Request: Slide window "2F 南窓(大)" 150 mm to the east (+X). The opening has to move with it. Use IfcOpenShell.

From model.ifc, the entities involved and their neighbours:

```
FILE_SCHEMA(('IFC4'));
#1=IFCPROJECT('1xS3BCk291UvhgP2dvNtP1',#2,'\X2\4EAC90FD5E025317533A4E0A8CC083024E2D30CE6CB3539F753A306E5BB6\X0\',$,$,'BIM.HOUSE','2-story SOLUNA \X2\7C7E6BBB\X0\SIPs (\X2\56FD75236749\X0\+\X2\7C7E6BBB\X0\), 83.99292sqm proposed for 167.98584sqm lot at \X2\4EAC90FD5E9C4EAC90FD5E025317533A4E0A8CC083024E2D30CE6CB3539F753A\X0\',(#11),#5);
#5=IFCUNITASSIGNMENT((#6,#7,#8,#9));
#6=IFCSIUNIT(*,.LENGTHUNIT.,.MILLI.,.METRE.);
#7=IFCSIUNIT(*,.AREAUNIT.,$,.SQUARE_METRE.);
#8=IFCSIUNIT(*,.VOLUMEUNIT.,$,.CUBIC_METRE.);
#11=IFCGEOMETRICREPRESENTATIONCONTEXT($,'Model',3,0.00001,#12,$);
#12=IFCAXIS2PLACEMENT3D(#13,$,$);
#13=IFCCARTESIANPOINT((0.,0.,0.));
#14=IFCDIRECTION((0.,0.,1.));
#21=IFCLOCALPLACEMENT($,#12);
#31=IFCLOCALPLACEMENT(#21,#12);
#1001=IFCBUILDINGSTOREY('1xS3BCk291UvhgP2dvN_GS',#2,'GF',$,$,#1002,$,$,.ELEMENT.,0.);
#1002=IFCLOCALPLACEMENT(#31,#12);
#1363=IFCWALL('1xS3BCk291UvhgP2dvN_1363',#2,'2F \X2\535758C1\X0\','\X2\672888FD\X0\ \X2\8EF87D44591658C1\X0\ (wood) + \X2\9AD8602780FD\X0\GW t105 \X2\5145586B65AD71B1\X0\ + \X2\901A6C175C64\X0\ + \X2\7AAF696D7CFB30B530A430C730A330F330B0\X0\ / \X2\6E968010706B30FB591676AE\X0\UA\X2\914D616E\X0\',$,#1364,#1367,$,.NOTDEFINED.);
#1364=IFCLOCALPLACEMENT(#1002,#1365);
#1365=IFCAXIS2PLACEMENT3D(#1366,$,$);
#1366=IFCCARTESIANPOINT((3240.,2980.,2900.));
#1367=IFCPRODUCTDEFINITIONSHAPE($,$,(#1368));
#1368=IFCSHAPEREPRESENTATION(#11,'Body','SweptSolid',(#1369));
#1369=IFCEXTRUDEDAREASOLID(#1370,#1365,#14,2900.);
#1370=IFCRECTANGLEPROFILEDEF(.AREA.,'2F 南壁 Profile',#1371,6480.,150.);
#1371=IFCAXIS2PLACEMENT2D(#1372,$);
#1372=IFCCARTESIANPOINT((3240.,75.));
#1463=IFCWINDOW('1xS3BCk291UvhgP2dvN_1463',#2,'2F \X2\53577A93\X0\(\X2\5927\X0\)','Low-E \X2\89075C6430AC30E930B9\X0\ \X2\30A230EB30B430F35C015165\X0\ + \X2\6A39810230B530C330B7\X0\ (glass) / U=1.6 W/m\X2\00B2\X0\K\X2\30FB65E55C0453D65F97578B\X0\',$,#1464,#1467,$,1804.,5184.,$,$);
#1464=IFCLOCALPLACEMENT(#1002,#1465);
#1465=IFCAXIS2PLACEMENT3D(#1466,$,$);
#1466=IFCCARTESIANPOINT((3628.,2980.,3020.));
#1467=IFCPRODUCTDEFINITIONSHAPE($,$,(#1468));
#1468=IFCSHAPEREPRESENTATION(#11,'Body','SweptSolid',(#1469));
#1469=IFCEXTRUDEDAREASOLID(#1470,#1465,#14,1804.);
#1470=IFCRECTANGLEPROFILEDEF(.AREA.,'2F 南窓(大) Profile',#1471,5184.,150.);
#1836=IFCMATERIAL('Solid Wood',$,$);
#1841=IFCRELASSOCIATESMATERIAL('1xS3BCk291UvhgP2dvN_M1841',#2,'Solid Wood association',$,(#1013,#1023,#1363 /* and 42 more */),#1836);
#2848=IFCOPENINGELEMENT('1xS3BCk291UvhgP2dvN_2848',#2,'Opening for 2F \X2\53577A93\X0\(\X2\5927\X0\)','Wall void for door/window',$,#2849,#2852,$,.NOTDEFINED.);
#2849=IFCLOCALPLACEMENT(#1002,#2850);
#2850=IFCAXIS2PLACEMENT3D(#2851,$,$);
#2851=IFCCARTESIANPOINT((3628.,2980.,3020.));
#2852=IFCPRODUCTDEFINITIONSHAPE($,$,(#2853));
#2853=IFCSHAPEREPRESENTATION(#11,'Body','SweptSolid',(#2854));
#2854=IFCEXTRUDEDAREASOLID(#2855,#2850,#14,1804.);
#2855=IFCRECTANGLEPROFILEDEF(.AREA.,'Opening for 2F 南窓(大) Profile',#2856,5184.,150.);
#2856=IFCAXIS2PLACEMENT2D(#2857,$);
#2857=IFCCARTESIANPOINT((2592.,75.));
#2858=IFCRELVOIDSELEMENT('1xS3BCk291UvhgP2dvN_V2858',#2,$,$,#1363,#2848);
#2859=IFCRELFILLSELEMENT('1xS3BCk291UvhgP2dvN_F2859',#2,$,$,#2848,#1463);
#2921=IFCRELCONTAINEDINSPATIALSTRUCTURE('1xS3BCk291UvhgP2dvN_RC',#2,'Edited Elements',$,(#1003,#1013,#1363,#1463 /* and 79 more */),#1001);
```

```python
import ifcopenshell
import ifcopenshell.api.geometry
import ifcopenshell.util.placement

model = ifcopenshell.open("model.ifc")

window = model.by_id(1463)
opening = window.FillsVoids[0].RelatingOpeningElement
wall = opening.VoidsElements[0].RelatingBuildingElement

wall_matrix = ifcopenshell.util.placement.get_local_placement(wall.ObjectPlacement)
shift = wall_matrix[:3, 0] * 150.0
before = ifcopenshell.util.placement.get_local_placement(window.ObjectPlacement)[:3, 3].copy()

# The window is not placed relative to its opening, so move both.
for product in (opening, window):
    matrix = ifcopenshell.util.placement.get_local_placement(product.ObjectPlacement)
    matrix[:3, 3] += shift
    ifcopenshell.api.geometry.edit_object_placement(model, product=product, matrix=matrix, is_si=False)

after = ifcopenshell.util.placement.get_local_placement(window.ObjectPlacement)[:3, 3]
print("window moved by", (after - before).round(3) + 0.0)

model.write("model-out.ifc")
```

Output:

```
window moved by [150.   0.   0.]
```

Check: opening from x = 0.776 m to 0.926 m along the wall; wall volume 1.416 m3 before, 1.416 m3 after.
